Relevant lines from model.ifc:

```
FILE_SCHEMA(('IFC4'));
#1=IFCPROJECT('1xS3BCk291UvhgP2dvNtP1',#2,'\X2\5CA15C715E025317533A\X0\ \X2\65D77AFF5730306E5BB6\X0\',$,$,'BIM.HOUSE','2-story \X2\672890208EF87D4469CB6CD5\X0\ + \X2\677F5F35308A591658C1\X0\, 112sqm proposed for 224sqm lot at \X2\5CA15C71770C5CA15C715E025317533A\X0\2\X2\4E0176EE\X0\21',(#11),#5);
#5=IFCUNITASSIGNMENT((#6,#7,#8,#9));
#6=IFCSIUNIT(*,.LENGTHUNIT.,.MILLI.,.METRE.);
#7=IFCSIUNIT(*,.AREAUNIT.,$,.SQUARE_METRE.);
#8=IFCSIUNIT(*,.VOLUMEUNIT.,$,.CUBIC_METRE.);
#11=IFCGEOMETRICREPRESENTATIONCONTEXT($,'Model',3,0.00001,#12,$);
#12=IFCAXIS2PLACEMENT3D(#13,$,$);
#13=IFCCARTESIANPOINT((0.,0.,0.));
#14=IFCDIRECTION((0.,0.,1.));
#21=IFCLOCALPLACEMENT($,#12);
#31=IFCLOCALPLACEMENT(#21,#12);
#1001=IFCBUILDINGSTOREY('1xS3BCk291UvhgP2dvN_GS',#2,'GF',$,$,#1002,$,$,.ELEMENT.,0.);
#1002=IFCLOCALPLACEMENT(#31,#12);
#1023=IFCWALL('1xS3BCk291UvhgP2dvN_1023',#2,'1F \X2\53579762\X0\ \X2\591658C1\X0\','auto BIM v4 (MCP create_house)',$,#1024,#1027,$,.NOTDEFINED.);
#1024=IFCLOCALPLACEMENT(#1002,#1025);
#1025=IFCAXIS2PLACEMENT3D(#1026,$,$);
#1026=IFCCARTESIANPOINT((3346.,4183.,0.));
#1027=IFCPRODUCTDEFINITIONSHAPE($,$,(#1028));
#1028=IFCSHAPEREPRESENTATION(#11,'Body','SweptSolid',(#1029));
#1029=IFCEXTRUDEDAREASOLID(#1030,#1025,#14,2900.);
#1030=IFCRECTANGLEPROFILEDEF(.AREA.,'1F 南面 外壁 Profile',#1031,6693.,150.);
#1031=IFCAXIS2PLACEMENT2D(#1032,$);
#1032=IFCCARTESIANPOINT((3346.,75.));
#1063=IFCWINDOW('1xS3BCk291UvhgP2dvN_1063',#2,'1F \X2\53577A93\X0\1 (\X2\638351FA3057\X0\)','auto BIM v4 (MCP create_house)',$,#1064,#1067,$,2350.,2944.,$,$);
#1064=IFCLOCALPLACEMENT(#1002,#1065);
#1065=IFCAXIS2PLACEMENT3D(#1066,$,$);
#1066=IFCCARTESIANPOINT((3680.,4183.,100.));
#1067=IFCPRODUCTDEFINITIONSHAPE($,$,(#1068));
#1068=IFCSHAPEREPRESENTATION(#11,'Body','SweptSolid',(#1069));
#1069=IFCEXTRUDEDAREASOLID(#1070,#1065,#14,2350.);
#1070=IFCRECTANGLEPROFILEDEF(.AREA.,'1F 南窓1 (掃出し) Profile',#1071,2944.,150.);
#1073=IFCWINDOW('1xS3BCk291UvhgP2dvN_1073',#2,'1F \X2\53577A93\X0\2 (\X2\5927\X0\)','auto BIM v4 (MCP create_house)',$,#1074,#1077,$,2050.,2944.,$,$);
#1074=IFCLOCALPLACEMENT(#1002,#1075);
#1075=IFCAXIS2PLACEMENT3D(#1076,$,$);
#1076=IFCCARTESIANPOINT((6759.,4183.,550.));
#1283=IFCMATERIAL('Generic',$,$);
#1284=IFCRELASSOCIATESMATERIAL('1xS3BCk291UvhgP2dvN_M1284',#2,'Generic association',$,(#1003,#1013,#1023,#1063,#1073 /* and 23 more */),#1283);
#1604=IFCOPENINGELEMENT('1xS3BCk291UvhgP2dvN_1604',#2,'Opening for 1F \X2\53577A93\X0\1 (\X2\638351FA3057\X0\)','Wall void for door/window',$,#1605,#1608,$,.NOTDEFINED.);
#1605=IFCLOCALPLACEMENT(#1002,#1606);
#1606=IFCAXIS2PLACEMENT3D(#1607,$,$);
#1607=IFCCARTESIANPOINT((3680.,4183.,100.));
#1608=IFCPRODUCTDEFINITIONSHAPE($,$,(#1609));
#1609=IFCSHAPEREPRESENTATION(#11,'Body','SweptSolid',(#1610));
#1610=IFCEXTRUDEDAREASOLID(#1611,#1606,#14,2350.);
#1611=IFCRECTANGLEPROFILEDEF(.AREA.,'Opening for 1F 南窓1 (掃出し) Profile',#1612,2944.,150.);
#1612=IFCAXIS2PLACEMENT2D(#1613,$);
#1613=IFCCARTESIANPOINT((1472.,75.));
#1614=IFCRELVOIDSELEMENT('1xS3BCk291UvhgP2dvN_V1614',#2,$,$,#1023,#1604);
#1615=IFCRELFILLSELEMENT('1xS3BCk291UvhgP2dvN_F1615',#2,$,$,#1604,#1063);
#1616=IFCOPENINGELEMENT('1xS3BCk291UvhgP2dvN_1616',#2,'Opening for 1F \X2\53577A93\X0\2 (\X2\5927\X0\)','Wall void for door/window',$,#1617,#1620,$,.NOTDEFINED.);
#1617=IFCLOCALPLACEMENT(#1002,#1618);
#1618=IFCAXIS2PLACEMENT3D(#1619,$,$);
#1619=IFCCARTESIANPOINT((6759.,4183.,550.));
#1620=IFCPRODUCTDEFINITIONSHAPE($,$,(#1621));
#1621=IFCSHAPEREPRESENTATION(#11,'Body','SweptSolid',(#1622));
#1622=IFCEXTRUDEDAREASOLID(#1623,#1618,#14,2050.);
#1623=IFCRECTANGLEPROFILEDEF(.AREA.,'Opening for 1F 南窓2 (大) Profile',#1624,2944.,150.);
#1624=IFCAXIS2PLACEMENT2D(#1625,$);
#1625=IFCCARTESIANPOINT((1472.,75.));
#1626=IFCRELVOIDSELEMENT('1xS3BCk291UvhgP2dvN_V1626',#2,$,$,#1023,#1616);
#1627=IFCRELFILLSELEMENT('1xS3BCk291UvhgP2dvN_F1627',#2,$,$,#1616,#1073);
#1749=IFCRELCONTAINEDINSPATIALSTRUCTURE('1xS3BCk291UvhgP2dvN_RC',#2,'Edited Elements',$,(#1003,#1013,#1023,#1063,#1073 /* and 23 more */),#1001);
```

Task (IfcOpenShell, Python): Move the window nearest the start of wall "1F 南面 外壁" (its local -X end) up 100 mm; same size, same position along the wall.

```python
import numpy as np
import ifcopenshell
import ifcopenshell.api.geometry
import ifcopenshell.util.placement
import ifcopenshell.util.unit

model = ifcopenshell.open("model.ifc")
unit_scale = ifcopenshell.util.unit.calculate_unit_scale(model)

window = model.by_guid("1xS3BCk291UvhgP2dvN_1063")
opening = window.FillsVoids[0].RelatingOpeningElement
dz = 100.0

shift = np.array([0.0, 0.0, dz])
# The window is not placed relative to its opening, so move both.
for product in (opening, window):
    matrix = ifcopenshell.util.placement.get_local_placement(product.ObjectPlacement)
    matrix[:3, 3] += shift
    ifcopenshell.api.geometry.edit_object_placement(model, product=product, matrix=matrix, is_si=False)

print(f"moved by {dz * unit_scale:+.3f} m")

model.write("model-out.ifc")
```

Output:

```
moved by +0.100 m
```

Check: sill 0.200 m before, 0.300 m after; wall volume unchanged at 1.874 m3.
